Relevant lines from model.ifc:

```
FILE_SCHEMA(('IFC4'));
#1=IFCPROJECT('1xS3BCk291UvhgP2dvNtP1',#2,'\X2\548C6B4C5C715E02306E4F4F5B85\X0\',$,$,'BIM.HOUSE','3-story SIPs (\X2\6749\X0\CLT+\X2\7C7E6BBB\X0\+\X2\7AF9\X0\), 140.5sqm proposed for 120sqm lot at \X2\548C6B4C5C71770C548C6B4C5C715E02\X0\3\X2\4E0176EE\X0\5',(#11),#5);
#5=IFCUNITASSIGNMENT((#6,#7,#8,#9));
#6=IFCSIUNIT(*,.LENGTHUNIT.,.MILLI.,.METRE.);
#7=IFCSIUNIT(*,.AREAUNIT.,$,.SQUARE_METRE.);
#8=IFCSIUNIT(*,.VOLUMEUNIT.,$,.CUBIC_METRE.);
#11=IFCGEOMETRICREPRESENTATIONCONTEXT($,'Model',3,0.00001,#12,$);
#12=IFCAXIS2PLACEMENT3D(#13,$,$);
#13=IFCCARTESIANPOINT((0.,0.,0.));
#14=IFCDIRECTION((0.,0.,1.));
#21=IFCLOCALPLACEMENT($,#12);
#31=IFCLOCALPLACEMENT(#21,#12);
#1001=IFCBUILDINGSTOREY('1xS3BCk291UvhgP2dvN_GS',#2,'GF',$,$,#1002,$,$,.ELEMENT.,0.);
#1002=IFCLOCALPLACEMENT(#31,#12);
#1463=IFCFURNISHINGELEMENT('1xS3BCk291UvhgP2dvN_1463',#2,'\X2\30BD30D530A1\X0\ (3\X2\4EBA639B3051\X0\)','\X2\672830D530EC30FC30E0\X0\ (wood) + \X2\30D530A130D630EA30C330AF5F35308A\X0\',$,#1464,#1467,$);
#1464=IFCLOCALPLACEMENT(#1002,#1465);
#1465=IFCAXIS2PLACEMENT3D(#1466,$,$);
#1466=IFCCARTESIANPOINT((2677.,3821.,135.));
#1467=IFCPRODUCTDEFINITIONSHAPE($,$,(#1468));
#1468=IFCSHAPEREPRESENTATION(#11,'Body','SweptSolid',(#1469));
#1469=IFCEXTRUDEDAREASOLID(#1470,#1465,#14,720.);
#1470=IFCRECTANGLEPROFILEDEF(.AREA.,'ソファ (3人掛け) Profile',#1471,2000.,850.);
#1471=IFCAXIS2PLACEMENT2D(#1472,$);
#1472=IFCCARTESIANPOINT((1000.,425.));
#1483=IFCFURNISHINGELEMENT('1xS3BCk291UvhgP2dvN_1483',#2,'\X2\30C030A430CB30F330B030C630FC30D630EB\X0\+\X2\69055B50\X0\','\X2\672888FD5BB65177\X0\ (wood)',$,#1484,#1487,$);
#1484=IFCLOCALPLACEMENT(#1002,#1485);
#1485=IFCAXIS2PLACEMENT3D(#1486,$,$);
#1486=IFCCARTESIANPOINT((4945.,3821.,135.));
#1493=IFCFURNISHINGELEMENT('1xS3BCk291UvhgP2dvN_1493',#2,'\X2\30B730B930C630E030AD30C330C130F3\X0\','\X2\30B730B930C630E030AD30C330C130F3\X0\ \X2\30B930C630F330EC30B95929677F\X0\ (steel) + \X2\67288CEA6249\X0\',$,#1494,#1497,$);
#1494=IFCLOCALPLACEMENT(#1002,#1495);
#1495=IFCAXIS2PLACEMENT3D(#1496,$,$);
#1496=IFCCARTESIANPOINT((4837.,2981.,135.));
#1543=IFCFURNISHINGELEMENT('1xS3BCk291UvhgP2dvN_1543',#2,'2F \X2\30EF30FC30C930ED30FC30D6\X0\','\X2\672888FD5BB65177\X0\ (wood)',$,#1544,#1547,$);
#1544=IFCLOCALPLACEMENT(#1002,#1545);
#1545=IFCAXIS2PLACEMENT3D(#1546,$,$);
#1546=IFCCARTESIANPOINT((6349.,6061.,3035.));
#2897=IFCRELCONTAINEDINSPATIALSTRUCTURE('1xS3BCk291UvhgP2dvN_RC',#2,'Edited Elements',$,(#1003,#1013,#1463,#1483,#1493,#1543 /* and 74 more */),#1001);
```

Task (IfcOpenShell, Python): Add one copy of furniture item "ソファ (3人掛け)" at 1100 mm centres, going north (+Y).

```python
import numpy as np
import ifcopenshell
import ifcopenshell.api.geometry
import ifcopenshell.api.root
import ifcopenshell.util.element
import ifcopenshell.util.placement
import ifcopenshell.util.unit

model = ifcopenshell.open("model.ifc")
unit_scale = ifcopenshell.util.unit.calculate_unit_scale(model)


def reuse_history(source, copy):
    """copy_class also copies each property set's owner history, people and application; keep the originals."""
    for rel in copy.IsDefinedBy:
        if rel.is_a("IfcRelDefinesByProperties") and (history := rel.RelatingPropertyDefinition.OwnerHistory):
            rel.RelatingPropertyDefinition.OwnerHistory = source.OwnerHistory
            ifcopenshell.util.element.remove_deep2(model, history)


source = model.by_id(1463)
base = ifcopenshell.util.placement.get_local_placement(source.ObjectPlacement)
step = np.array([0.0, 1.0, 0.0]) * 1.1 / unit_scale

for i in range(1, 2):
    copy = ifcopenshell.api.root.copy_class(model, product=source)
    copy.Representation = ifcopenshell.util.element.copy_deep(
        model, source.Representation, exclude=["IfcGeometricRepresentationContext", "IfcRepresentationMap"]
    )
    reuse_history(source, copy)
    matrix = base.copy()
    matrix[:3, 3] += i * step
    print("added at", matrix[:3, 3].round(3) + 0.0)
    ifcopenshell.api.geometry.edit_object_placement(model, product=copy, matrix=matrix, is_si=False)

model.write("model_edited.ifc")
```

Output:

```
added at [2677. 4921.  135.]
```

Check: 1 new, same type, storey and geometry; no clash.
